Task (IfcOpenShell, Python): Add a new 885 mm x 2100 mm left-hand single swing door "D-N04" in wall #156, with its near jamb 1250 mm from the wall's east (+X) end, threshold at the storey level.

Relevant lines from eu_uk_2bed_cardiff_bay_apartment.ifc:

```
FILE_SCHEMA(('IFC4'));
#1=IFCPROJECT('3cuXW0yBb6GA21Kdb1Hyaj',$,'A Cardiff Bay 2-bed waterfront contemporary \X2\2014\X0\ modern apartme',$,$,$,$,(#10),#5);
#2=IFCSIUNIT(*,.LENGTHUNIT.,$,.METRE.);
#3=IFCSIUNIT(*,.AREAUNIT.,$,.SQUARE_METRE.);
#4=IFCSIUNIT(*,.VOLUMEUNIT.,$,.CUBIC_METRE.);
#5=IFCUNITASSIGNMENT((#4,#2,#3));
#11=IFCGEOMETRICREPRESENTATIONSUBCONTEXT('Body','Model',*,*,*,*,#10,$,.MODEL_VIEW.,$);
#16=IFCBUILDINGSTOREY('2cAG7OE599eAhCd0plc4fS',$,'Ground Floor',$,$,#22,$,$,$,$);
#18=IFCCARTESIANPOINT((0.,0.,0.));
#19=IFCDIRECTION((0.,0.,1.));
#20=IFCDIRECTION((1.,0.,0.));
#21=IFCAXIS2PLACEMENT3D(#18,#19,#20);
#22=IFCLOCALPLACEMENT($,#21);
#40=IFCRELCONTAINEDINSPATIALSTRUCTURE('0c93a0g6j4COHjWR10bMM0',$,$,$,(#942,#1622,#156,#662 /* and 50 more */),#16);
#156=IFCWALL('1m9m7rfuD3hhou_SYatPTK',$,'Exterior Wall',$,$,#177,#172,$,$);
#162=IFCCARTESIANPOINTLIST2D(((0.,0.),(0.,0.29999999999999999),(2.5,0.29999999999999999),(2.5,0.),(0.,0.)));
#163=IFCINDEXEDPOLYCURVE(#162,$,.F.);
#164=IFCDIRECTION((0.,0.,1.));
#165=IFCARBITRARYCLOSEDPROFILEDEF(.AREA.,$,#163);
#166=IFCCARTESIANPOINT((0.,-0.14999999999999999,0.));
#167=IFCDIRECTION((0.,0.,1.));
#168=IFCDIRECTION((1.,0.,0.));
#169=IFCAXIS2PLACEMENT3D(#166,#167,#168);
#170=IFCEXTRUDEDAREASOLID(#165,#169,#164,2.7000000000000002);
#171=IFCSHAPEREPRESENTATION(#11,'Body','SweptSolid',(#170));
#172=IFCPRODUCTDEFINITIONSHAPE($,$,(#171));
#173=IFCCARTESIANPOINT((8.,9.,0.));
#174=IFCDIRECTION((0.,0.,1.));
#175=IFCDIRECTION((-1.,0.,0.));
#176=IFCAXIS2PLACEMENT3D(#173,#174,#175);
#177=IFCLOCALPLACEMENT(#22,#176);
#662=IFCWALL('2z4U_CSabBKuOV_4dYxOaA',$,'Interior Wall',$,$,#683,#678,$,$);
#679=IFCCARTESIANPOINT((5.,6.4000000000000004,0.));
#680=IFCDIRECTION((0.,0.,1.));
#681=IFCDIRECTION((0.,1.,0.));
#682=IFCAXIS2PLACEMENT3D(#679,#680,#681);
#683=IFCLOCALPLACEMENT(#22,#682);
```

```python
import numpy as np
import ifcopenshell
import ifcopenshell.api.feature
import ifcopenshell.api.geometry
import ifcopenshell.api.root
import ifcopenshell.api.spatial
import ifcopenshell.geom
import ifcopenshell.util.element
import ifcopenshell.util.placement
import ifcopenshell.util.representation
import ifcopenshell.util.shape
import ifcopenshell.util.unit

model = ifcopenshell.open("eu_uk_2bed_cardiff_bay_apartment.ifc")
unit_scale = ifcopenshell.util.unit.calculate_unit_scale(model)
settings = ifcopenshell.geom.settings()


def volume(element):
    """Net volume in cubic metres, openings subtracted."""
    shape = ifcopenshell.geom.create_shape(settings, element)
    return ifcopenshell.util.shape.get_volume(shape.geometry)


wall = model.by_id(156)
storey = ifcopenshell.util.element.get_container(wall, ifc_class="IfcBuildingStorey")
context = ifcopenshell.util.representation.get_context(model, "Model", "Body", "MODEL_VIEW")
before = volume(wall)

width, height, from_end, sill = 0.885, 2.1, 1.25, 0.0  # metres

# The wall runs along its own X axis, and the end named is its -X end.
wall_shape = ifcopenshell.geom.create_shape(settings, wall)
x, y, z = ifcopenshell.util.shape.get_vertices(wall_shape.geometry).T
start = x.min() + from_end
face, thickness = float(y.min()), float(y.max() - y.min())
wall_matrix = ifcopenshell.util.placement.get_local_placement(wall.ObjectPlacement)
level = ifcopenshell.util.placement.get_local_placement(storey.ObjectPlacement)[2, 3]


def in_wall(x, y):
    """Placement at x, y metres in the wall's axes, at sill height."""
    matrix = wall_matrix.copy()
    matrix[:, 3] = wall_matrix @ np.array([x / unit_scale, y / unit_scale, 0.0, 1.0])
    matrix[2, 3] = level + sill / unit_scale
    return matrix


# Opening: a box that overshoots both wall faces by 50 mm.
opening = ifcopenshell.api.root.create_entity(model, ifc_class="IfcOpeningElement", predefined_type="OPENING")
box = ifcopenshell.api.geometry.add_wall_representation(
    model, context=context, length=width, height=height, thickness=thickness + 0.1
)
ifcopenshell.api.geometry.assign_representation(model, product=opening, representation=box)
ifcopenshell.api.geometry.edit_object_placement(model, product=opening, matrix=in_wall(start, face - 0.05), is_si=False)
ifcopenshell.api.feature.add_feature(model, feature=opening, element=wall)

door = ifcopenshell.api.root.create_entity(model, ifc_class="IfcDoor", name="D-N04", predefined_type="DOOR")
door.OverallWidth, door.OverallHeight = width / unit_scale, height / unit_scale
door.OperationType = "SINGLE_SWING_LEFT"
body = ifcopenshell.api.geometry.add_door_representation(
    model,
    context=context,
    overall_width=door.OverallWidth,
    overall_height=door.OverallHeight,
    operation_type="SINGLE_SWING_LEFT",
    lining_properties={"LiningDepth": thickness / unit_scale, "ThresholdDepth": thickness / unit_scale},
)
ifcopenshell.api.geometry.assign_representation(model, product=door, representation=body)
ifcopenshell.api.spatial.assign_container(model, products=[door], relating_structure=storey)
ifcopenshell.api.feature.add_filling(model, opening=opening, element=door)

# The lining spans the wall, so the door starts at the wall face.
ifcopenshell.api.geometry.edit_object_placement(model, product=door, matrix=in_wall(start, face), is_si=False)

after = volume(wall)

print(f"wall volume {before:.3f} -> {after:.3f} m3")

model.write("eu_uk_2bed_cardiff_bay_apartment_v2.ifc")
```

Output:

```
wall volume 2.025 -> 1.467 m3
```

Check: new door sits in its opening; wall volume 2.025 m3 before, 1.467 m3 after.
